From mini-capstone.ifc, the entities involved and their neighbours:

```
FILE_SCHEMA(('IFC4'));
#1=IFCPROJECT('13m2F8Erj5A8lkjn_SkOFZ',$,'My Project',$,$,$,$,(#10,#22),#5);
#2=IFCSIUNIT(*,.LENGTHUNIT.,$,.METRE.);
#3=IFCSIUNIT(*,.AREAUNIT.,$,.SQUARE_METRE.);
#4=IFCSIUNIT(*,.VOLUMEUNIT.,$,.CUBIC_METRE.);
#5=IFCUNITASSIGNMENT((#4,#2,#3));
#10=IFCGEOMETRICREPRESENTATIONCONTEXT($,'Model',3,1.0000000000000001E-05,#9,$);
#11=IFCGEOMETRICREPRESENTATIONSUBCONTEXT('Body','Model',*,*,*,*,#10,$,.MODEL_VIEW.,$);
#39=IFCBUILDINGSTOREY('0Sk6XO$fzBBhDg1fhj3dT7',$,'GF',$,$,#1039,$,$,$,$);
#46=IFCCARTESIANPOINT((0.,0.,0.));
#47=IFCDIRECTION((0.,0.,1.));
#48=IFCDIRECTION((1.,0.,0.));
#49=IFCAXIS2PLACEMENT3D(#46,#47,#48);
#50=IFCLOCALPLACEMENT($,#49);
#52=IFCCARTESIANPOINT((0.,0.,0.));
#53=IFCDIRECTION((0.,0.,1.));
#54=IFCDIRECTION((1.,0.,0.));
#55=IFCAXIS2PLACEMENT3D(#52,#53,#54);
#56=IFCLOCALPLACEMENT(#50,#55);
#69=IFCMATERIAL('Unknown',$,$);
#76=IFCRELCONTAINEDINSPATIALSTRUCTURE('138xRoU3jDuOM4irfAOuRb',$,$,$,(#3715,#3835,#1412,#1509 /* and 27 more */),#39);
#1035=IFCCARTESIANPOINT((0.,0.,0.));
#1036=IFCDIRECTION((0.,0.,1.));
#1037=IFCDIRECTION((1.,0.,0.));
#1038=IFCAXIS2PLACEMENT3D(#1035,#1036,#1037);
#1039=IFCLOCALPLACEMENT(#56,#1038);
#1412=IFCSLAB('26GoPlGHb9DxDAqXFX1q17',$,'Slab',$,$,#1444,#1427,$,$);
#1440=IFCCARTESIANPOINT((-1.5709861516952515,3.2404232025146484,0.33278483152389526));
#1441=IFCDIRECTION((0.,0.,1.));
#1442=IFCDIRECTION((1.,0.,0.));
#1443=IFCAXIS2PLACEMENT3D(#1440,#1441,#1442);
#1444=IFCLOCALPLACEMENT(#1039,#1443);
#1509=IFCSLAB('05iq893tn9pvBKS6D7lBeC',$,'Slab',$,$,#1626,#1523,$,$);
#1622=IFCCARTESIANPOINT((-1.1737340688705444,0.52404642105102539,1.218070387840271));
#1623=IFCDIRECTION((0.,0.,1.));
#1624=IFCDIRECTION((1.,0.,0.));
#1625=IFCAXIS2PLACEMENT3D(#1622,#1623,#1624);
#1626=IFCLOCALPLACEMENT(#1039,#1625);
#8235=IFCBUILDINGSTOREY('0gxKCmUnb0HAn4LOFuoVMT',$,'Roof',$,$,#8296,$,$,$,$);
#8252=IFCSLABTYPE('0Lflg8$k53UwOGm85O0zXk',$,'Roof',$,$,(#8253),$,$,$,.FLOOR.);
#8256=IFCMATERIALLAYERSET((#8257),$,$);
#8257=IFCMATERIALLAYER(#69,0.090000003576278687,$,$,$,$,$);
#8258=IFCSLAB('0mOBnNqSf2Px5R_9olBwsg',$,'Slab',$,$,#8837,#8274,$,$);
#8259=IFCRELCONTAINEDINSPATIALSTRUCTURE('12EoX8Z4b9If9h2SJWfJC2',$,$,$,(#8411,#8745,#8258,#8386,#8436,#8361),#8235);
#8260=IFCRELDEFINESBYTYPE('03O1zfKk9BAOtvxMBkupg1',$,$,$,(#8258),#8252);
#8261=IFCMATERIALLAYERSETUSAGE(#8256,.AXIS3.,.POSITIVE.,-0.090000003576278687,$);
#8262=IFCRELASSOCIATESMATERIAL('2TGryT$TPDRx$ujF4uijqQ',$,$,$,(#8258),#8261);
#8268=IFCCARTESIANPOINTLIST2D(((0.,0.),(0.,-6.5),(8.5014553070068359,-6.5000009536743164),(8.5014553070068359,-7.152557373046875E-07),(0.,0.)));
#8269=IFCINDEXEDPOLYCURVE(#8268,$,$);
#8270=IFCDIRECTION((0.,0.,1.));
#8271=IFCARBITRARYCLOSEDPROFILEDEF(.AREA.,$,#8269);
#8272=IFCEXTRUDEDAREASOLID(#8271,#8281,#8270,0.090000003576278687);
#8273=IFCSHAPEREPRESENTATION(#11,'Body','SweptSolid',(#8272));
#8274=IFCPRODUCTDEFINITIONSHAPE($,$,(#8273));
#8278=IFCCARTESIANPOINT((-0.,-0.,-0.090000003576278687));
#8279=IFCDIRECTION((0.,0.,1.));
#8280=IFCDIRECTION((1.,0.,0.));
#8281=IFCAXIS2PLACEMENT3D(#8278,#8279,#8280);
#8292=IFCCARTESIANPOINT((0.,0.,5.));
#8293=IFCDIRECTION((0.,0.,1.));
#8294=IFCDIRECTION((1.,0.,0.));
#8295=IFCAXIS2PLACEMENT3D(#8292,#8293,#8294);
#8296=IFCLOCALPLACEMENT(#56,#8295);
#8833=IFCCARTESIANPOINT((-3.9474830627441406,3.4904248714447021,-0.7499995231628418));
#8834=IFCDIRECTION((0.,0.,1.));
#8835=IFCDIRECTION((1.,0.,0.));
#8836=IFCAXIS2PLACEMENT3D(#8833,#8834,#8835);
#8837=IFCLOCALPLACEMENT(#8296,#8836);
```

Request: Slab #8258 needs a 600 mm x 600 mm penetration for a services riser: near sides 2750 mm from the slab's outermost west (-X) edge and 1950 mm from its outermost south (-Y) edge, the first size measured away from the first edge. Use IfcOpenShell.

```python
import numpy as np
import ifcopenshell
import ifcopenshell.api.feature
import ifcopenshell.api.geometry
import ifcopenshell.api.root
import ifcopenshell.geom
import ifcopenshell.util.placement
import ifcopenshell.util.representation
import ifcopenshell.util.shape
import ifcopenshell.util.unit

model = ifcopenshell.open("mini-capstone.ifc")
unit_scale = ifcopenshell.util.unit.calculate_unit_scale(model)
settings = ifcopenshell.geom.settings()


def volume(element):
    """Net volume in cubic metres, openings subtracted."""
    shape = ifcopenshell.geom.create_shape(settings, element)
    return ifcopenshell.util.shape.get_volume(shape.geometry)


slab = model.by_id(8258)
before = volume(slab)

# Extent in the slab's own axes, in metres. The edges named are its -X and -Y sides.
slab_shape = ifcopenshell.geom.create_shape(settings, slab)
vertices = ifcopenshell.util.shape.get_vertices(slab_shape.geometry)
x_min, y_min, bottom = vertices.min(axis=0)
top = vertices[:, 2].max()

opening = ifcopenshell.api.root.create_entity(model, ifc_class="IfcOpeningElement", name="Services riser opening", predefined_type="OPENING")
context = ifcopenshell.util.representation.get_context(model, "Model", "Body", "MODEL_VIEW")
width, depth = 0.6, 0.6
outline = [(0.0, 0.0), (width, 0.0), (width, depth), (0.0, depth), (0.0, 0.0)]
# Overshoot both faces by 50 mm so the cut is clean.
shape = ifcopenshell.api.geometry.add_slab_representation(
    model, context=context, depth=top - bottom + 0.1, polyline=outline
)
ifcopenshell.api.geometry.assign_representation(model, product=opening, representation=shape)

matrix = ifcopenshell.util.placement.get_local_placement(slab.ObjectPlacement)
matrix[:, 3] = matrix @ np.append(np.array([x_min + 2.75, y_min + 1.95, bottom - 0.05]) / unit_scale, 1.0)
ifcopenshell.api.geometry.edit_object_placement(model, product=opening, matrix=matrix, is_si=False)
ifcopenshell.api.feature.add_feature(model, feature=opening, element=slab)

after = volume(slab)

print(f"slab volume {before:.3f} -> {after:.3f} m3")

model.write("mini-capstone_edited.ifc")
```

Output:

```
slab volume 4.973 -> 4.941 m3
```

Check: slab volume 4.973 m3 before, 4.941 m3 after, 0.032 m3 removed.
